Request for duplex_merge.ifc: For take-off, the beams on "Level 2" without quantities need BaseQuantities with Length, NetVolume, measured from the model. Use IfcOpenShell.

First a look at what the model holds.

```python
import ifcopenshell
import ifcopenshell.util.element
import ifcopenshell.util.unit

model = ifcopenshell.open("duplex_merge.ifc")
print(model.schema)
for unit_type in ("LENGTHUNIT", "AREAUNIT", "VOLUMEUNIT"):
    print(unit_type, ifcopenshell.util.unit.calculate_unit_scale(model, unit_type))
storey = next(s for s in model.by_type("IfcBuildingStorey") if s.Name == "Level 2")
beams = [e for e in ifcopenshell.util.element.get_decomposition(storey) if e.is_a("IfcBeam")]
for e in sorted(beams, key=lambda e: e.id()):
    print(e.id(), e.is_a(), e.Name, list(ifcopenshell.util.element.get_psets(e, qtos_only=True)), sep=" | ")
```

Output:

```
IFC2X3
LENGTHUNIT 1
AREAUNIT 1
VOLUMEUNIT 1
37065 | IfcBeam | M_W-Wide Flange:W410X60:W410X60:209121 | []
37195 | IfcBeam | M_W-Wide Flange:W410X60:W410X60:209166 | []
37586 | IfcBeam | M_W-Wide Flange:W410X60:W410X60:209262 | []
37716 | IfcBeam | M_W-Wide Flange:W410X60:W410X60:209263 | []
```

```python
import ifcopenshell
import ifcopenshell.api.pset
import ifcopenshell.geom
import ifcopenshell.util.element
import ifcopenshell.util.shape
import ifcopenshell.util.unit

model = ifcopenshell.open("duplex_merge.ifc")
unit_scale = ifcopenshell.util.unit.calculate_unit_scale(model)
volume_scale = ifcopenshell.util.unit.calculate_unit_scale(model, "VOLUMEUNIT")
settings = ifcopenshell.geom.settings()

storey = next(s for s in model.by_type("IfcBuildingStorey") if s.Name == "Level 2")
beams = [e for e in ifcopenshell.util.element.get_decomposition(storey) if e.is_a("IfcBeam")]

for e in sorted(beams, key=lambda e: e.id()):
    if ifcopenshell.util.element.get_psets(e, qtos_only=True, should_inherit=False):
        continue
    # Geometry comes back in metres, in the element's own axes.
    shape = ifcopenshell.geom.create_shape(settings, e)
    values = {
        "Length": ifcopenshell.util.shape.get_max_xyz(shape.geometry) / unit_scale,
        "NetVolume": ifcopenshell.util.shape.get_volume(shape.geometry) / volume_scale,
    }
    qto = ifcopenshell.api.pset.add_qto(model, product=e, name="BaseQuantities")
    ifcopenshell.api.pset.edit_qto(model, qto=qto, properties=values)
    print(e.id(), {k: round(v, 3) for k, v in values.items()})

model.write("duplex_merge_updated.ifc")
```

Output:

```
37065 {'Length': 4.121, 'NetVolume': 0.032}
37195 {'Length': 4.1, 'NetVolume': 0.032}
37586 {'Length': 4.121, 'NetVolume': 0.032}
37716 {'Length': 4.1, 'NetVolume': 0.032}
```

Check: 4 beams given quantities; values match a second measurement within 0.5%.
